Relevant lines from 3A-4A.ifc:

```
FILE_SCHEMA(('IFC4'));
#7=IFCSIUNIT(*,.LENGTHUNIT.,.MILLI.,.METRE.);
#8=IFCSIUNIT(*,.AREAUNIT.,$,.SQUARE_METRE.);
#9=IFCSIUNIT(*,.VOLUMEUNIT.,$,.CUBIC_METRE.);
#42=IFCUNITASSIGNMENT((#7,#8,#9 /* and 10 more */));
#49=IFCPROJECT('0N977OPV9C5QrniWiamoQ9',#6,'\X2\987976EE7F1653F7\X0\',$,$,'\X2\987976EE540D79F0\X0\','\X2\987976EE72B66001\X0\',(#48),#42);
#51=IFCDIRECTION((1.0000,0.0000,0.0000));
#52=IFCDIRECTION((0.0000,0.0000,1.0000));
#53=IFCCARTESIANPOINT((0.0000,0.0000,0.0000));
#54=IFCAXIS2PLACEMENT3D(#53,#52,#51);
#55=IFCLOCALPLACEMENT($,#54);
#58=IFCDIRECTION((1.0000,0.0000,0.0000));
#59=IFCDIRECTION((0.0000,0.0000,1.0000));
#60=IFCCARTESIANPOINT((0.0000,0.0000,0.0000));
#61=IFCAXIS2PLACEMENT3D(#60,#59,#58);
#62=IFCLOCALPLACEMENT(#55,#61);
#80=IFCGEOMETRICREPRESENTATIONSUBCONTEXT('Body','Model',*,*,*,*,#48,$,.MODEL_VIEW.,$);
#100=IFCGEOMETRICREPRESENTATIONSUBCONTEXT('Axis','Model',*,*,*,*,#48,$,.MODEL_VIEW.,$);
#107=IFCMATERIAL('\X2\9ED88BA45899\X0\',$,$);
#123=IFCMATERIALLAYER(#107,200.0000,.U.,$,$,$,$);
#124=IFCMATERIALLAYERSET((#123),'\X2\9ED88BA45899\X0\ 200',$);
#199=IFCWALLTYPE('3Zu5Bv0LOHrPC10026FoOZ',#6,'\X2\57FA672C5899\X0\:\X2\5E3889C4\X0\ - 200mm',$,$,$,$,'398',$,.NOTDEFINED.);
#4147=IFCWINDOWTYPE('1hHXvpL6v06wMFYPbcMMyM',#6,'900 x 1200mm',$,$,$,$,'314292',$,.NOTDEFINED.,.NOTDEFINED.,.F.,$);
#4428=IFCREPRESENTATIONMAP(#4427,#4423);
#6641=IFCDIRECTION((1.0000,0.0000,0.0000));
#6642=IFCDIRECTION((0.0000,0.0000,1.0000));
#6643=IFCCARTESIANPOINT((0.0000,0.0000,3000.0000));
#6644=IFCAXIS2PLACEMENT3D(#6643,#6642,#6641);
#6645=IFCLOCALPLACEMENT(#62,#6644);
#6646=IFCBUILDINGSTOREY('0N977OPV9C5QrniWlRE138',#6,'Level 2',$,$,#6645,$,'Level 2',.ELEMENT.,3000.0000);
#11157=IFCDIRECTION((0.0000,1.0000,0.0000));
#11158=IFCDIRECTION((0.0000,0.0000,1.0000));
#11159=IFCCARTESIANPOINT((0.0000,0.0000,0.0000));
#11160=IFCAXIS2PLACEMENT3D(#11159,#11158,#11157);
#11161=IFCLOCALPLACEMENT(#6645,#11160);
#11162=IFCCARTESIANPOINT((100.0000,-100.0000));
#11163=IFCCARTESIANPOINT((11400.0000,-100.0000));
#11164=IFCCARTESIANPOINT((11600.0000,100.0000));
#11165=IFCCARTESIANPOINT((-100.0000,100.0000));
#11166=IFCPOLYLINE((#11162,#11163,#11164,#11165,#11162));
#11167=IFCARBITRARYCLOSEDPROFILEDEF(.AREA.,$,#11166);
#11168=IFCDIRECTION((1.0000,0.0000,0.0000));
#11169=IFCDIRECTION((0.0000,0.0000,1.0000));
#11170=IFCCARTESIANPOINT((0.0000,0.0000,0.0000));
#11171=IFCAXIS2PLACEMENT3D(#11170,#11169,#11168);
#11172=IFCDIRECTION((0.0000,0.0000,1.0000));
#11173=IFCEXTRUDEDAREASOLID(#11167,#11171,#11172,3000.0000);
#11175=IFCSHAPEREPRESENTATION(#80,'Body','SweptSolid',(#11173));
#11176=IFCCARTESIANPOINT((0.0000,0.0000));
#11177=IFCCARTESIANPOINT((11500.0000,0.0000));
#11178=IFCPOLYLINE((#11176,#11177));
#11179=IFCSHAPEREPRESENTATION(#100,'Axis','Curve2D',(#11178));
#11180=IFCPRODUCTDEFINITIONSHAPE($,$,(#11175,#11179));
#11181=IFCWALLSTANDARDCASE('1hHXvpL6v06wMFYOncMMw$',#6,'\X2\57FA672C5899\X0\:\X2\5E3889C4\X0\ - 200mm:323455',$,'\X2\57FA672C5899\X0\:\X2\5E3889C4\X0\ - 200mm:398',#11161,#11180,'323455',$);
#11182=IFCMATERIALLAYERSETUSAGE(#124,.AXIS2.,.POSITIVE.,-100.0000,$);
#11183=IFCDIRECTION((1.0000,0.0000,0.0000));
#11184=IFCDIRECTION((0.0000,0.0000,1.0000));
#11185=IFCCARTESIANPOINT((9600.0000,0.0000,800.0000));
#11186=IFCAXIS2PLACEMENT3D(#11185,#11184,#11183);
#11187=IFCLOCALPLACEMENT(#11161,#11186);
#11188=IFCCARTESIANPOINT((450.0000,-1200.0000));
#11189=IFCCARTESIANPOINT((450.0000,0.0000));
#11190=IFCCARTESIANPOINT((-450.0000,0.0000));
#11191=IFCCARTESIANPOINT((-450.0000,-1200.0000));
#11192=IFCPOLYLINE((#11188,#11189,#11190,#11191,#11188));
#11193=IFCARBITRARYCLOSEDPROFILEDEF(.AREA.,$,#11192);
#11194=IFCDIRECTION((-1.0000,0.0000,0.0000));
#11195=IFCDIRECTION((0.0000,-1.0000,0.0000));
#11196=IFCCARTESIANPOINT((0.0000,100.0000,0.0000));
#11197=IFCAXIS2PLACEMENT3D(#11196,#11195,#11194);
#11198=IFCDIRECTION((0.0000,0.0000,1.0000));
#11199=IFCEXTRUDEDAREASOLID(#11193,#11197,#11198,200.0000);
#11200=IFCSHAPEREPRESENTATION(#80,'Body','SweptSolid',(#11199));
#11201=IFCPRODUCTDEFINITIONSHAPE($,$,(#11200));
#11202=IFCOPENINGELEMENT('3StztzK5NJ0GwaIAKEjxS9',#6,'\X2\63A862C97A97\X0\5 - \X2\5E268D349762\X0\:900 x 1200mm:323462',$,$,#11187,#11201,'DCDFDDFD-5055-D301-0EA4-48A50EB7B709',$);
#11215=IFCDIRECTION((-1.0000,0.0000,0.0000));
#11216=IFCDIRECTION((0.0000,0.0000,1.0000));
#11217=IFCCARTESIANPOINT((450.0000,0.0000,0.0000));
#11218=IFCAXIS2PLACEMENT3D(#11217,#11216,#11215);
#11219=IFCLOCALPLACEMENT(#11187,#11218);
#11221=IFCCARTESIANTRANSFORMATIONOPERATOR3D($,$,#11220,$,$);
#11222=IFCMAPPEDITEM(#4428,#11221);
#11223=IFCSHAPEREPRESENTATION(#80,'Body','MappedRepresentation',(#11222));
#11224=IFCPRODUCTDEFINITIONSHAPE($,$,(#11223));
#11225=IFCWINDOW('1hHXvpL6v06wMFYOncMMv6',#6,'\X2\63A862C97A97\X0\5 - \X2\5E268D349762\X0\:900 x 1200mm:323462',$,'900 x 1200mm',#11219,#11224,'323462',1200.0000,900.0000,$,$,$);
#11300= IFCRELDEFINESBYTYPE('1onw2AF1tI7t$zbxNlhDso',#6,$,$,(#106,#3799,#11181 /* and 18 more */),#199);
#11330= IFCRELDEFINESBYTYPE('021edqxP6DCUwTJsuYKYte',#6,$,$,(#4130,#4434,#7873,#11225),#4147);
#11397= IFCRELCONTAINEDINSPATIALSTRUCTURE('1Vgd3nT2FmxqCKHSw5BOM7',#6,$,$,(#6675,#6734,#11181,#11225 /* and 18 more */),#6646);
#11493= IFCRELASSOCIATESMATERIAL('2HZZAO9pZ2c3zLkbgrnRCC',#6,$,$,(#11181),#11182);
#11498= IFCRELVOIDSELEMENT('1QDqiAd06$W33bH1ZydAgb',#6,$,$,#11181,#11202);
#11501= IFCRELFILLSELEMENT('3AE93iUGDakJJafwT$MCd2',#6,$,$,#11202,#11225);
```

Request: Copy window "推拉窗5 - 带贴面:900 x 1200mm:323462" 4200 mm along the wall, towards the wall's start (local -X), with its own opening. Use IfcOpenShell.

```python
import ifcopenshell
import ifcopenshell.api.feature
import ifcopenshell.api.geometry
import ifcopenshell.api.root
import ifcopenshell.geom
import ifcopenshell.util.element
import ifcopenshell.util.placement
import ifcopenshell.util.shape
import ifcopenshell.util.unit

model = ifcopenshell.open("3A-4A.ifc")
unit_scale = ifcopenshell.util.unit.calculate_unit_scale(model)
settings = ifcopenshell.geom.settings()


def volume(element):
    """Net volume in cubic metres, openings subtracted."""
    shape = ifcopenshell.geom.create_shape(settings, element)
    return ifcopenshell.util.shape.get_volume(shape.geometry)


def reuse_history(source, copy):
    """copy_class also copies each property set's owner history, people and application; keep the originals."""
    for rel in copy.IsDefinedBy:
        if rel.is_a("IfcRelDefinesByProperties") and (history := rel.RelatingPropertyDefinition.OwnerHistory):
            rel.RelatingPropertyDefinition.OwnerHistory = source.OwnerHistory
            ifcopenshell.util.element.remove_deep2(model, history)


window = model.by_guid("1hHXvpL6v06wMFYOncMMv6")
opening = window.FillsVoids[0].RelatingOpeningElement
wall = opening.VoidsElements[0].RelatingBuildingElement
before = volume(wall)
shift = ifcopenshell.util.placement.get_local_placement(wall.ObjectPlacement)[:3, 0] * -4.2 / unit_scale

# copy_class copies the void relationship, type, container and properties, but no geometry.
new_opening = ifcopenshell.api.root.copy_class(model, product=opening)
new_opening.Representation = ifcopenshell.util.element.copy_deep(
    model, opening.Representation, exclude=["IfcGeometricRepresentationContext", "IfcRepresentationMap"]
)
new_opening.Name = "推拉窗5 - 带贴面:900 x 1200mm"
new_opening.Tag = None
new_window = ifcopenshell.api.root.copy_class(model, product=window)
new_window.Representation = ifcopenshell.util.element.copy_deep(
    model, window.Representation, exclude=["IfcGeometricRepresentationContext", "IfcRepresentationMap"]
)
new_window.Name = "推拉窗5 - 带贴面:900 x 1200mm"
new_window.Tag = None
reuse_history(window, new_window)
ifcopenshell.api.feature.add_filling(model, opening=new_opening, element=new_window)

for old, new in ((opening, new_opening), (window, new_window)):
    matrix = ifcopenshell.util.placement.get_local_placement(old.ObjectPlacement)
    matrix[:3, 3] += shift
    ifcopenshell.api.geometry.edit_object_placement(model, product=new, matrix=matrix, is_si=False)

after = volume(wall)

print(f"wall volume {before:.3f} -> {after:.3f} m3")

model.write("3A-4A_updated.ifc")
```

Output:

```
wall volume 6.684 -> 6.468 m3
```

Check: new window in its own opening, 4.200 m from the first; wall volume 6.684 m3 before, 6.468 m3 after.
